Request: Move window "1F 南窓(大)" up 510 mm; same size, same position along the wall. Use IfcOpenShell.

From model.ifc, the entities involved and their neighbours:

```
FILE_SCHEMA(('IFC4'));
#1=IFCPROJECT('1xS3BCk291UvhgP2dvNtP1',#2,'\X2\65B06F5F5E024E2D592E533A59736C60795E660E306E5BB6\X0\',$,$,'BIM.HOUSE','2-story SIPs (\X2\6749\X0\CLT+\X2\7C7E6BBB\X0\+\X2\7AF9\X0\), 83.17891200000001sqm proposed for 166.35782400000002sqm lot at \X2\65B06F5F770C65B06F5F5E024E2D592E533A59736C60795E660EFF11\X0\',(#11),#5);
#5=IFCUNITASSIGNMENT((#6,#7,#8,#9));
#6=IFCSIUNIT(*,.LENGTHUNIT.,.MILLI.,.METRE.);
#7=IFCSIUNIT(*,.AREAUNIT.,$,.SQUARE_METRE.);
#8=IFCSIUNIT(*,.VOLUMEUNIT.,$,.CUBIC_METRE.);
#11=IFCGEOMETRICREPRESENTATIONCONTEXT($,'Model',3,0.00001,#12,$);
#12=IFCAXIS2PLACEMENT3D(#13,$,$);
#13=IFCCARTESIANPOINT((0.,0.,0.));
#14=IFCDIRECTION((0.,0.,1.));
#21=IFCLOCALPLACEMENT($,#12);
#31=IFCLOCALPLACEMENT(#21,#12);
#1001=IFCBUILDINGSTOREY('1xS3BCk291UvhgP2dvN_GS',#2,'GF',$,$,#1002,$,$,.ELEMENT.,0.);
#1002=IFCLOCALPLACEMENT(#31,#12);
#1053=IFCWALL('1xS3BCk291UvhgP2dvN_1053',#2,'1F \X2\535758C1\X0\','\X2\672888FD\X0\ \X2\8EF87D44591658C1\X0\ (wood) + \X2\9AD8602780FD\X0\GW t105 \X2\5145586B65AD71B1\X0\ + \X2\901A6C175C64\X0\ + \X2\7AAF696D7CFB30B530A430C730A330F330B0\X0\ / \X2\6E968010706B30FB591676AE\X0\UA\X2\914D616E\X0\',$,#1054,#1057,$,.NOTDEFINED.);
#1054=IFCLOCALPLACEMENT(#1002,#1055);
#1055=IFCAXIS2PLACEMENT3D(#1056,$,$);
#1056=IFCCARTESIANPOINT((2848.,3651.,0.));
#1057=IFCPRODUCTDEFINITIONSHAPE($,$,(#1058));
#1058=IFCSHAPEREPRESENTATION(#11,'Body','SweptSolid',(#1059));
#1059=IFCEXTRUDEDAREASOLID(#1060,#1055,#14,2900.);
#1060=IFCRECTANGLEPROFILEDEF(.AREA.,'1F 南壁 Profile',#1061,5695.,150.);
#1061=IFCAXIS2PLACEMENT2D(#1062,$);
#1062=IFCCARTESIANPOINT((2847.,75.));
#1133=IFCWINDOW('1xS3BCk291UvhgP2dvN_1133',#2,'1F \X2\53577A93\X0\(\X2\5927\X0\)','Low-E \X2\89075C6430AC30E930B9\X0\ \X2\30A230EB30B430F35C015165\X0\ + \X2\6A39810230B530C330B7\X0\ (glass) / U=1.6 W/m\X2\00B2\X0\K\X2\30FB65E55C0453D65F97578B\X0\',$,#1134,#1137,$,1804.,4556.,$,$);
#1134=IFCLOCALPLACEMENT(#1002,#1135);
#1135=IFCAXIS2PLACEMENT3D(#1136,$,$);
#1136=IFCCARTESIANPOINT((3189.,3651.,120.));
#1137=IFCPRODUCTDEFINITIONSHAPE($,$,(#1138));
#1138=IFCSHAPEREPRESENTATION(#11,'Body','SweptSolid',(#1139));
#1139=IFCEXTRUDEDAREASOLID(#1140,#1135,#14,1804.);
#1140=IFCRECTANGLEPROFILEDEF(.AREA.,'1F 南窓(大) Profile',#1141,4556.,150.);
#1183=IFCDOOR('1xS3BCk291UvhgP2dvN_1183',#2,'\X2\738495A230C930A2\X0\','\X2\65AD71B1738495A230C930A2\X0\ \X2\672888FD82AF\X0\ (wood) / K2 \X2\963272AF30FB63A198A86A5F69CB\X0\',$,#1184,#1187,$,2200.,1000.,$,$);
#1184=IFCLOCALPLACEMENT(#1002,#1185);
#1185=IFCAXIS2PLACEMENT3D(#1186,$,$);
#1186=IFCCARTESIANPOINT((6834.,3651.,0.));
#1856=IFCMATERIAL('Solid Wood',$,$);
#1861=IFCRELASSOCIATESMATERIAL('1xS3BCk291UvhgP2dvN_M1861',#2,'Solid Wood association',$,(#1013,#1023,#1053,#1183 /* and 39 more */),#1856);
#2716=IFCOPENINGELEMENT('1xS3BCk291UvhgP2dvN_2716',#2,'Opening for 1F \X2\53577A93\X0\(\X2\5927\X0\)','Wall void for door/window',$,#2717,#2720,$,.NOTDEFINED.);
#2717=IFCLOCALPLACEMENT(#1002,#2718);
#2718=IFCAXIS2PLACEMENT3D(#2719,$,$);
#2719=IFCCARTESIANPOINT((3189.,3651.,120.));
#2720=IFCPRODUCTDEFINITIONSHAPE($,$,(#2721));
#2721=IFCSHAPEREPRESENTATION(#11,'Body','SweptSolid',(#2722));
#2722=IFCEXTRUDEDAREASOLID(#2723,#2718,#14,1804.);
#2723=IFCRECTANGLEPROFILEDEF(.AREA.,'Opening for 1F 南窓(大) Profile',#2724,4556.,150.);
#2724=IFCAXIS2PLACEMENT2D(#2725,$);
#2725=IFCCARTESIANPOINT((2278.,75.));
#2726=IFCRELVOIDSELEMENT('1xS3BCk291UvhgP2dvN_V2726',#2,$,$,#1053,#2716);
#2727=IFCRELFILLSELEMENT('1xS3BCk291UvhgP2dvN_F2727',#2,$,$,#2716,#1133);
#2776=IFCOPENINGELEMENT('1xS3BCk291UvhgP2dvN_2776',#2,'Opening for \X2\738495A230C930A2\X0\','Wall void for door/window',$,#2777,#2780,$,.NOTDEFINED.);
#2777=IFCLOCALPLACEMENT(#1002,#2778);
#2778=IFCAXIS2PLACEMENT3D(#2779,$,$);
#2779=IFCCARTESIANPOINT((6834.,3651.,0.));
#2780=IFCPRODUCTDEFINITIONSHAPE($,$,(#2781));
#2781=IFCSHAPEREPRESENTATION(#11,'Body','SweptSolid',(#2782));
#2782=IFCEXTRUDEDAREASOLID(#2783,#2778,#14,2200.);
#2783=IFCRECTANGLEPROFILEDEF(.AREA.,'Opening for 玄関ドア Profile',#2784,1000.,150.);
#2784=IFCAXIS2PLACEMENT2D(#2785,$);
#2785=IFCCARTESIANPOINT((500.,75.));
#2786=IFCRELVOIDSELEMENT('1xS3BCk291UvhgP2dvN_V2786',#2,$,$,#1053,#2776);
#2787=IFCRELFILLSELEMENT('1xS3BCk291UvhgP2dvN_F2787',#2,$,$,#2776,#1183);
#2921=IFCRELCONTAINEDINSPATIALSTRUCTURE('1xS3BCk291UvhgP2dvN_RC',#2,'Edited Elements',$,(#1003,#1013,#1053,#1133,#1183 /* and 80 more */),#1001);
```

```python
import numpy as np
import ifcopenshell
import ifcopenshell.api.geometry
import ifcopenshell.util.placement
import ifcopenshell.util.unit

model = ifcopenshell.open("model.ifc")
unit_scale = ifcopenshell.util.unit.calculate_unit_scale(model)

window = model.by_guid("1xS3BCk291UvhgP2dvN_1133")
opening = window.FillsVoids[0].RelatingOpeningElement
dz = 0.51 / unit_scale

shift = np.array([0.0, 0.0, dz])
# The window is not placed relative to its opening, so move both.
for product in (opening, window):
    matrix = ifcopenshell.util.placement.get_local_placement(product.ObjectPlacement)
    matrix[:3, 3] += shift
    ifcopenshell.api.geometry.edit_object_placement(model, product=product, matrix=matrix, is_si=False)

print(f"moved by {dz * unit_scale:+.3f} m")

model.write("model_edited.ifc")
```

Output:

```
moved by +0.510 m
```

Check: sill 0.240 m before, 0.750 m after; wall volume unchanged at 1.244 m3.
